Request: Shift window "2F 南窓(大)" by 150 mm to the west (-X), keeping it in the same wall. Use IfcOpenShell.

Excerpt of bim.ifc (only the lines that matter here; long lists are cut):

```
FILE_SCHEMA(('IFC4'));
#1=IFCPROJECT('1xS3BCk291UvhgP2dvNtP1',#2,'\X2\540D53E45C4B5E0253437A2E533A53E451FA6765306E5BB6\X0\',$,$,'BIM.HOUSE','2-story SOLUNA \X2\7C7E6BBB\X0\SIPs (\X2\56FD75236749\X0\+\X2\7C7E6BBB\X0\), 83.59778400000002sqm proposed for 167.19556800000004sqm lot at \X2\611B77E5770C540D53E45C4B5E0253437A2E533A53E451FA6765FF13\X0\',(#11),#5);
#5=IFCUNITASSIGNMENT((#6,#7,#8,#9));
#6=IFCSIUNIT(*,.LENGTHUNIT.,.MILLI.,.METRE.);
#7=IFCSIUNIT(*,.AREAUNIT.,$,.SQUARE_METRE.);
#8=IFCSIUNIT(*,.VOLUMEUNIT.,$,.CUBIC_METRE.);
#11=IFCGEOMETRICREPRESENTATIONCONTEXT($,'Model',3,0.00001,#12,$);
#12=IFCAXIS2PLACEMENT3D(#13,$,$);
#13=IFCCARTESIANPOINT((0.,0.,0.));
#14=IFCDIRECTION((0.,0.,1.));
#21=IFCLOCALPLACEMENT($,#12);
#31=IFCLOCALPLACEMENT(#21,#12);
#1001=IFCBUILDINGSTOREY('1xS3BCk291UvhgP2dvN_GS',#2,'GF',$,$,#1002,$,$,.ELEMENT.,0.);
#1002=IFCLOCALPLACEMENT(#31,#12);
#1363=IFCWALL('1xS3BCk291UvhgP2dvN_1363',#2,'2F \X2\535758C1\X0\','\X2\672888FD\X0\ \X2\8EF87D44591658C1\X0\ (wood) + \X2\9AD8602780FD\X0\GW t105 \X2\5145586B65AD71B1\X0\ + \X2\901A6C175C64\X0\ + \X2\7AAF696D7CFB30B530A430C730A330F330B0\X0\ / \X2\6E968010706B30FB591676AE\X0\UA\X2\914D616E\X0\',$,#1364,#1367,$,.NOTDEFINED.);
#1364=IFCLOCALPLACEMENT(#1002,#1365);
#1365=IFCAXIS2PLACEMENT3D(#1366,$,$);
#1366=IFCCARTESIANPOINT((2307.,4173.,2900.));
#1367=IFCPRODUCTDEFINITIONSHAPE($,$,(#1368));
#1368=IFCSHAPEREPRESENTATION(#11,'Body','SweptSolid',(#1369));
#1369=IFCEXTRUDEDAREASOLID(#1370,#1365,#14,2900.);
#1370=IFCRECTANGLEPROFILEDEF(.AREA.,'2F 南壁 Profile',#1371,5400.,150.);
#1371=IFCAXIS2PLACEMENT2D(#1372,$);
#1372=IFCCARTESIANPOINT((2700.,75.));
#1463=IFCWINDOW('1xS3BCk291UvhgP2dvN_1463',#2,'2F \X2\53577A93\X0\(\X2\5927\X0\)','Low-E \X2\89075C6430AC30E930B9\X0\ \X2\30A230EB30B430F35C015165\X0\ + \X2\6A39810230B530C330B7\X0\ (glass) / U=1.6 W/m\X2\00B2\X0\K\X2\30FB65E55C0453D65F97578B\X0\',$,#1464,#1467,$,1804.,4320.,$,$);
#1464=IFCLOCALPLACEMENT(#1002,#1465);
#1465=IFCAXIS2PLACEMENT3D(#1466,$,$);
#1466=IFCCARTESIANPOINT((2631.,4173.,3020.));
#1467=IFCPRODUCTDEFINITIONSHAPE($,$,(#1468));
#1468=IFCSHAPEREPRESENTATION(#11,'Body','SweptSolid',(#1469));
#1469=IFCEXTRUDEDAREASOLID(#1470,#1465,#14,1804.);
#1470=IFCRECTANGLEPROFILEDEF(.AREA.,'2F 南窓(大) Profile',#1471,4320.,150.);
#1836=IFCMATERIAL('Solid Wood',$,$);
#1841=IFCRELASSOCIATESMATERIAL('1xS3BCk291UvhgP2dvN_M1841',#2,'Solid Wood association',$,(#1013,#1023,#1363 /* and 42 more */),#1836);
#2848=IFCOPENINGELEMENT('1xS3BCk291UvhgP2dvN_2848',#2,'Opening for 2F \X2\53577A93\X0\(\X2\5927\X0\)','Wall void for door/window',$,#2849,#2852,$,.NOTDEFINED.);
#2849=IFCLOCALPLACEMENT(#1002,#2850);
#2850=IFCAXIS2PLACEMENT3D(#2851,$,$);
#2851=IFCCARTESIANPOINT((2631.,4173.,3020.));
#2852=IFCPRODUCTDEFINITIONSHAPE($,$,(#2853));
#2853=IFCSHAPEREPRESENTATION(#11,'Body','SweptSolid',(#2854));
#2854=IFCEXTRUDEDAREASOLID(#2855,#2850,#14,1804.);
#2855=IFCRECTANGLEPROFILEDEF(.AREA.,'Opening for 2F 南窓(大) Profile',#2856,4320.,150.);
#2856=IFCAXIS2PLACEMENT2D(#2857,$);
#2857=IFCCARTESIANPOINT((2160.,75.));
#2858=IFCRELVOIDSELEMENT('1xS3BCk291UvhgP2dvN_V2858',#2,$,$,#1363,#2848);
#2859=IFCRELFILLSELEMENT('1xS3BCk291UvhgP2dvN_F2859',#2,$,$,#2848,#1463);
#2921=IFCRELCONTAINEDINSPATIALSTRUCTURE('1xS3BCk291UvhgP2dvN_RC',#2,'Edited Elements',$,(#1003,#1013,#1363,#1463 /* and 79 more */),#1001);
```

```python
import ifcopenshell
import ifcopenshell.api.geometry
import ifcopenshell.util.placement

model = ifcopenshell.open("bim.ifc")

window = model.by_guid("1xS3BCk291UvhgP2dvN_1463")
opening = window.FillsVoids[0].RelatingOpeningElement
wall = opening.VoidsElements[0].RelatingBuildingElement

wall_matrix = ifcopenshell.util.placement.get_local_placement(wall.ObjectPlacement)
shift = wall_matrix[:3, 0] * -150.0
before = ifcopenshell.util.placement.get_local_placement(window.ObjectPlacement)[:3, 3].copy()

# The window is not placed relative to its opening, so move both.
for product in (opening, window):
    matrix = ifcopenshell.util.placement.get_local_placement(product.ObjectPlacement)
    matrix[:3, 3] += shift
    ifcopenshell.api.geometry.edit_object_placement(model, product=product, matrix=matrix, is_si=False)

after = ifcopenshell.util.placement.get_local_placement(window.ObjectPlacement)[:3, 3]
print("window moved by", (after - before).round(3) + 0.0)

model.write("bim_edited.ifc")
```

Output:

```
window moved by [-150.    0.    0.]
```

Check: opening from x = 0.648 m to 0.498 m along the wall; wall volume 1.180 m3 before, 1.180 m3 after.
